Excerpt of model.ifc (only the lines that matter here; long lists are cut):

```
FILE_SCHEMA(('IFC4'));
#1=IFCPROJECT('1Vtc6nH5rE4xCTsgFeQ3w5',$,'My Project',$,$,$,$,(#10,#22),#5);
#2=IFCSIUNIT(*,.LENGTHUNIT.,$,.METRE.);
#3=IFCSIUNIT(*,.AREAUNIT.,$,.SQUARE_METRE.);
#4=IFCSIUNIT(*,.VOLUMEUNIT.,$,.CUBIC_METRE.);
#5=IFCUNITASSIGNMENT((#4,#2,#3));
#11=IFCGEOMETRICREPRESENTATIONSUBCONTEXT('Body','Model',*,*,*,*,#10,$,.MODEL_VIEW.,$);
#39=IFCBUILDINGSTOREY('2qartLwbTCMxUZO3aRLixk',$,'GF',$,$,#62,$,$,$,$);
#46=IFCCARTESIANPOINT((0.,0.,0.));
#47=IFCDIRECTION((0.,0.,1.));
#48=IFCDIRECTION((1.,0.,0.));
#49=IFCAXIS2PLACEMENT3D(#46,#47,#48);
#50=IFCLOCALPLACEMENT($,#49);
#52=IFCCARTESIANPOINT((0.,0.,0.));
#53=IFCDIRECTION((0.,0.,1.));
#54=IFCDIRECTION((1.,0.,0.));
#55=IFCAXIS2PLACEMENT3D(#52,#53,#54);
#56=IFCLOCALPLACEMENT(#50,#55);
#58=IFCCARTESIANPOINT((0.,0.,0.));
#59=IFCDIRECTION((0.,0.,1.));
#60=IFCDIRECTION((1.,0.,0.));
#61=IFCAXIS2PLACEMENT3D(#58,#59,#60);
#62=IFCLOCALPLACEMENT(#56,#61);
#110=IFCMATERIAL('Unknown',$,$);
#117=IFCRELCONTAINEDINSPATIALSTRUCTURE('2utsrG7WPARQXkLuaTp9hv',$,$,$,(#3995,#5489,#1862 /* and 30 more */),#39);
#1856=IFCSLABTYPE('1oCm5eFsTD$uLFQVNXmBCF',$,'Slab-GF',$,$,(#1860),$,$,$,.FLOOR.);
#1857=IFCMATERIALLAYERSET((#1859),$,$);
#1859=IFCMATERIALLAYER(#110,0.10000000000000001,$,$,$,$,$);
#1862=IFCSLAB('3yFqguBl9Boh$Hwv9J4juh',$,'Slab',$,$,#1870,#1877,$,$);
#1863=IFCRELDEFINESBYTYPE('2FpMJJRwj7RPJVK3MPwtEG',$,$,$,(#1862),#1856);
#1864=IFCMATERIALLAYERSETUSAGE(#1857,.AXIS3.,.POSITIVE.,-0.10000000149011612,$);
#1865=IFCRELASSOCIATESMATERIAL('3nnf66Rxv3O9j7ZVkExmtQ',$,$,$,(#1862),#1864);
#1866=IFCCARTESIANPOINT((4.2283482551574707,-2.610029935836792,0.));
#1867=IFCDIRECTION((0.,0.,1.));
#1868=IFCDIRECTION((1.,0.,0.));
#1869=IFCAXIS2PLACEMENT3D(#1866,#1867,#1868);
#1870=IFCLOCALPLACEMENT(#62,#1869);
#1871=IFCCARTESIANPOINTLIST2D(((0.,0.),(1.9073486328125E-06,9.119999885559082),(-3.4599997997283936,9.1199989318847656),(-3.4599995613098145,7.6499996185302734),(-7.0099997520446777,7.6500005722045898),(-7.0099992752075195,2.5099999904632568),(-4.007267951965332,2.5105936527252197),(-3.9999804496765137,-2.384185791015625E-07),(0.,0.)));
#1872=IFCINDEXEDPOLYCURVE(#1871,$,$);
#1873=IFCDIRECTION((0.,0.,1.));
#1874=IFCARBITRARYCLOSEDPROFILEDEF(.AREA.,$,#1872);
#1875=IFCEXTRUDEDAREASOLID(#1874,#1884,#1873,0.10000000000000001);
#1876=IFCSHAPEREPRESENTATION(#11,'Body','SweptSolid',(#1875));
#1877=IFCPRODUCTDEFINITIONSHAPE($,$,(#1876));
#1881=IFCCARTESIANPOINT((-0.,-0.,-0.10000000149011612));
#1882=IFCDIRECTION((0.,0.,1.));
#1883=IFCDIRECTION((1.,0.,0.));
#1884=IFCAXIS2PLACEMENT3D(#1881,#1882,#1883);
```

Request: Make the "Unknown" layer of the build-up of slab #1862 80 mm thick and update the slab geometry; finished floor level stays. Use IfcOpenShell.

```python
import ifcopenshell
import ifcopenshell.util.element
import ifcopenshell.util.representation
import ifcopenshell.util.unit

model = ifcopenshell.open("model.ifc")
unit_scale = ifcopenshell.util.unit.calculate_unit_scale(model)

layer_set = model.by_id(1857)
layer = next(l for l in layer_set.MaterialLayers if l.Material and l.Material.Name == "Unknown")
change = 0.08 / unit_scale - layer.LayerThickness
layer.LayerThickness += change

# Geometry does not follow the layer set by itself.
slabs = [e for e in ifcopenshell.util.element.get_elements_by_material(model, layer_set) if e.is_a("IfcSlab")]
for slab in sorted(slabs, key=lambda e: e.id()):
    body = ifcopenshell.util.representation.get_representation(slab, "Model", "Body")
    solid = body.Items[0]
    old_depth = solid.Depth
    solid.Depth += change
    # Extruded upwards: lower the start of the extrusion so the top stays.
    x, y, z = solid.Position.Location.Coordinates
    solid.Position.Location = model.createIfcCartesianPoint((x, y, z - change))
    print(slab.id(), f"{old_depth:g} -> {solid.Depth:g}")

# The layers are counted up from the underside, which has moved.
for usage in {ifcopenshell.util.element.get_material(slab) for slab in slabs}:
    usage.OffsetFromReferenceLine -= change

model.write("model_updated.ifc")
```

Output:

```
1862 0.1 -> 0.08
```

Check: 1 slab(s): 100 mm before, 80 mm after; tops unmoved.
